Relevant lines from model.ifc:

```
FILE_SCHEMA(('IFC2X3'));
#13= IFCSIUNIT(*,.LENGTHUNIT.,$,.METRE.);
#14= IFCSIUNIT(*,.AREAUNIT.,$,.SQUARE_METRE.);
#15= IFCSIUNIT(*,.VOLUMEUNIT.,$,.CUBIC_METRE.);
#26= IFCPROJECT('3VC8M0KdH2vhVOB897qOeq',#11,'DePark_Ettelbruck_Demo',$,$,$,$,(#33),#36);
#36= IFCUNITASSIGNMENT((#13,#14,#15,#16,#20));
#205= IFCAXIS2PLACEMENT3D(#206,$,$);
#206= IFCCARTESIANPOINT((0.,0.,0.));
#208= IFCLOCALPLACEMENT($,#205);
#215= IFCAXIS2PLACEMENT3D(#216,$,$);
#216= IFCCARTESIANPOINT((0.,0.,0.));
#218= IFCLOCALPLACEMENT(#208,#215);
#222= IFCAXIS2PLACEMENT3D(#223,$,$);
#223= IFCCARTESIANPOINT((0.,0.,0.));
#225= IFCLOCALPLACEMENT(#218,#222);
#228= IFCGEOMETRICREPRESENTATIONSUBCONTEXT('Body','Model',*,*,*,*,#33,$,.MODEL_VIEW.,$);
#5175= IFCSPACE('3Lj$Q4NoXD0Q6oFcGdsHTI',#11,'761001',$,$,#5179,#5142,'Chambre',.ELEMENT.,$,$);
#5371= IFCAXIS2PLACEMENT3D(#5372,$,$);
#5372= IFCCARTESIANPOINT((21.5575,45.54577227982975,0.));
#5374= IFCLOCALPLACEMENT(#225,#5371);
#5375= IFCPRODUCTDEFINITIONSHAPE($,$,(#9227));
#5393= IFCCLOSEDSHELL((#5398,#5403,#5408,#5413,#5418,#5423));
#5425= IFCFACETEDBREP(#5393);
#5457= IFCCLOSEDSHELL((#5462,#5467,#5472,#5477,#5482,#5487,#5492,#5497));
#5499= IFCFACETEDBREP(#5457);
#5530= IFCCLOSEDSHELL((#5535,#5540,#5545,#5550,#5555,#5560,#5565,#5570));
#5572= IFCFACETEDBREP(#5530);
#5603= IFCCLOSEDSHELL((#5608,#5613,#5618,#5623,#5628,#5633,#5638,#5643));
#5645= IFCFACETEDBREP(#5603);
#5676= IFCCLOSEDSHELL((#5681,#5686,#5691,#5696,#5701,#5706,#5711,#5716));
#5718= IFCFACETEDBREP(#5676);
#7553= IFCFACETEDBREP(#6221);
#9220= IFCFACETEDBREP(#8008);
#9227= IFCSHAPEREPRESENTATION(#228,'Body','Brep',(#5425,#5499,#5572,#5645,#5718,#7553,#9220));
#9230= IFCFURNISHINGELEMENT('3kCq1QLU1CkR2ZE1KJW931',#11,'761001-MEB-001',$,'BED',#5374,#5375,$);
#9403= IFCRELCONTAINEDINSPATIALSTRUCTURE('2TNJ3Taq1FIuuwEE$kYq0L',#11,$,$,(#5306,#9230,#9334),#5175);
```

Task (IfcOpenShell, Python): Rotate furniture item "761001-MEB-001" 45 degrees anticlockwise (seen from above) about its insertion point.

```python
import ifcopenshell
import ifcopenshell.api.geometry
import ifcopenshell.util.placement

model = ifcopenshell.open("model.ifc")

item = model.by_id(9230)
matrix = ifcopenshell.util.placement.get_local_placement(item.ObjectPlacement)
matrix = matrix @ ifcopenshell.util.placement.rotation(45, "Z")
ifcopenshell.api.geometry.edit_object_placement(model, product=item, matrix=matrix, is_si=False)

print(ifcopenshell.util.placement.get_local_placement(item.ObjectPlacement).round(3) + 0.0)

model.write("model_rev.ifc")
```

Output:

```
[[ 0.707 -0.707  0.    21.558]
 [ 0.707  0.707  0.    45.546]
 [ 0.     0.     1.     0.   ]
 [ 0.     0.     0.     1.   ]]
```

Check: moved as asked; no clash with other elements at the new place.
